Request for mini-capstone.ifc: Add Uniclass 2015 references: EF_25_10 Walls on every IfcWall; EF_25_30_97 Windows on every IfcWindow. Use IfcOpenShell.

First a look at what the model holds.

```python
import ifcopenshell

model = ifcopenshell.open("mini-capstone.ifc")
print(model.schema)
print("classifications:", [c.Name for c in model.by_type("IfcClassification")])
for ifc_class in ("IfcDoor", "IfcRoof", "IfcStair", "IfcWall", "IfcWindow"):
    print(ifc_class, len(model.by_type(ifc_class)))
```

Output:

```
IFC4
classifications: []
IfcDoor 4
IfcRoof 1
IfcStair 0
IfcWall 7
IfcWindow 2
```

```python
import ifcopenshell
import ifcopenshell.api.classification

model = ifcopenshell.open("mini-capstone.ifc")

system = ifcopenshell.api.classification.add_classification(model, classification="Uniclass 2015")

codes = {
    "IfcWall": ("EF_25_10", "Walls"),
    "IfcWindow": ("EF_25_30_97", "Windows"),
}
for ifc_class, (code, name) in codes.items():
    products = model.by_type(ifc_class)
    ifcopenshell.api.classification.add_reference(
        model, products=products, classification=system, identification=code, name=name
    )
    print(code, len(products))

model.write("mini-capstone_edited.ifc")
```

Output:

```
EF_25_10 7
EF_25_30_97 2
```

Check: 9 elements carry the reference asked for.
